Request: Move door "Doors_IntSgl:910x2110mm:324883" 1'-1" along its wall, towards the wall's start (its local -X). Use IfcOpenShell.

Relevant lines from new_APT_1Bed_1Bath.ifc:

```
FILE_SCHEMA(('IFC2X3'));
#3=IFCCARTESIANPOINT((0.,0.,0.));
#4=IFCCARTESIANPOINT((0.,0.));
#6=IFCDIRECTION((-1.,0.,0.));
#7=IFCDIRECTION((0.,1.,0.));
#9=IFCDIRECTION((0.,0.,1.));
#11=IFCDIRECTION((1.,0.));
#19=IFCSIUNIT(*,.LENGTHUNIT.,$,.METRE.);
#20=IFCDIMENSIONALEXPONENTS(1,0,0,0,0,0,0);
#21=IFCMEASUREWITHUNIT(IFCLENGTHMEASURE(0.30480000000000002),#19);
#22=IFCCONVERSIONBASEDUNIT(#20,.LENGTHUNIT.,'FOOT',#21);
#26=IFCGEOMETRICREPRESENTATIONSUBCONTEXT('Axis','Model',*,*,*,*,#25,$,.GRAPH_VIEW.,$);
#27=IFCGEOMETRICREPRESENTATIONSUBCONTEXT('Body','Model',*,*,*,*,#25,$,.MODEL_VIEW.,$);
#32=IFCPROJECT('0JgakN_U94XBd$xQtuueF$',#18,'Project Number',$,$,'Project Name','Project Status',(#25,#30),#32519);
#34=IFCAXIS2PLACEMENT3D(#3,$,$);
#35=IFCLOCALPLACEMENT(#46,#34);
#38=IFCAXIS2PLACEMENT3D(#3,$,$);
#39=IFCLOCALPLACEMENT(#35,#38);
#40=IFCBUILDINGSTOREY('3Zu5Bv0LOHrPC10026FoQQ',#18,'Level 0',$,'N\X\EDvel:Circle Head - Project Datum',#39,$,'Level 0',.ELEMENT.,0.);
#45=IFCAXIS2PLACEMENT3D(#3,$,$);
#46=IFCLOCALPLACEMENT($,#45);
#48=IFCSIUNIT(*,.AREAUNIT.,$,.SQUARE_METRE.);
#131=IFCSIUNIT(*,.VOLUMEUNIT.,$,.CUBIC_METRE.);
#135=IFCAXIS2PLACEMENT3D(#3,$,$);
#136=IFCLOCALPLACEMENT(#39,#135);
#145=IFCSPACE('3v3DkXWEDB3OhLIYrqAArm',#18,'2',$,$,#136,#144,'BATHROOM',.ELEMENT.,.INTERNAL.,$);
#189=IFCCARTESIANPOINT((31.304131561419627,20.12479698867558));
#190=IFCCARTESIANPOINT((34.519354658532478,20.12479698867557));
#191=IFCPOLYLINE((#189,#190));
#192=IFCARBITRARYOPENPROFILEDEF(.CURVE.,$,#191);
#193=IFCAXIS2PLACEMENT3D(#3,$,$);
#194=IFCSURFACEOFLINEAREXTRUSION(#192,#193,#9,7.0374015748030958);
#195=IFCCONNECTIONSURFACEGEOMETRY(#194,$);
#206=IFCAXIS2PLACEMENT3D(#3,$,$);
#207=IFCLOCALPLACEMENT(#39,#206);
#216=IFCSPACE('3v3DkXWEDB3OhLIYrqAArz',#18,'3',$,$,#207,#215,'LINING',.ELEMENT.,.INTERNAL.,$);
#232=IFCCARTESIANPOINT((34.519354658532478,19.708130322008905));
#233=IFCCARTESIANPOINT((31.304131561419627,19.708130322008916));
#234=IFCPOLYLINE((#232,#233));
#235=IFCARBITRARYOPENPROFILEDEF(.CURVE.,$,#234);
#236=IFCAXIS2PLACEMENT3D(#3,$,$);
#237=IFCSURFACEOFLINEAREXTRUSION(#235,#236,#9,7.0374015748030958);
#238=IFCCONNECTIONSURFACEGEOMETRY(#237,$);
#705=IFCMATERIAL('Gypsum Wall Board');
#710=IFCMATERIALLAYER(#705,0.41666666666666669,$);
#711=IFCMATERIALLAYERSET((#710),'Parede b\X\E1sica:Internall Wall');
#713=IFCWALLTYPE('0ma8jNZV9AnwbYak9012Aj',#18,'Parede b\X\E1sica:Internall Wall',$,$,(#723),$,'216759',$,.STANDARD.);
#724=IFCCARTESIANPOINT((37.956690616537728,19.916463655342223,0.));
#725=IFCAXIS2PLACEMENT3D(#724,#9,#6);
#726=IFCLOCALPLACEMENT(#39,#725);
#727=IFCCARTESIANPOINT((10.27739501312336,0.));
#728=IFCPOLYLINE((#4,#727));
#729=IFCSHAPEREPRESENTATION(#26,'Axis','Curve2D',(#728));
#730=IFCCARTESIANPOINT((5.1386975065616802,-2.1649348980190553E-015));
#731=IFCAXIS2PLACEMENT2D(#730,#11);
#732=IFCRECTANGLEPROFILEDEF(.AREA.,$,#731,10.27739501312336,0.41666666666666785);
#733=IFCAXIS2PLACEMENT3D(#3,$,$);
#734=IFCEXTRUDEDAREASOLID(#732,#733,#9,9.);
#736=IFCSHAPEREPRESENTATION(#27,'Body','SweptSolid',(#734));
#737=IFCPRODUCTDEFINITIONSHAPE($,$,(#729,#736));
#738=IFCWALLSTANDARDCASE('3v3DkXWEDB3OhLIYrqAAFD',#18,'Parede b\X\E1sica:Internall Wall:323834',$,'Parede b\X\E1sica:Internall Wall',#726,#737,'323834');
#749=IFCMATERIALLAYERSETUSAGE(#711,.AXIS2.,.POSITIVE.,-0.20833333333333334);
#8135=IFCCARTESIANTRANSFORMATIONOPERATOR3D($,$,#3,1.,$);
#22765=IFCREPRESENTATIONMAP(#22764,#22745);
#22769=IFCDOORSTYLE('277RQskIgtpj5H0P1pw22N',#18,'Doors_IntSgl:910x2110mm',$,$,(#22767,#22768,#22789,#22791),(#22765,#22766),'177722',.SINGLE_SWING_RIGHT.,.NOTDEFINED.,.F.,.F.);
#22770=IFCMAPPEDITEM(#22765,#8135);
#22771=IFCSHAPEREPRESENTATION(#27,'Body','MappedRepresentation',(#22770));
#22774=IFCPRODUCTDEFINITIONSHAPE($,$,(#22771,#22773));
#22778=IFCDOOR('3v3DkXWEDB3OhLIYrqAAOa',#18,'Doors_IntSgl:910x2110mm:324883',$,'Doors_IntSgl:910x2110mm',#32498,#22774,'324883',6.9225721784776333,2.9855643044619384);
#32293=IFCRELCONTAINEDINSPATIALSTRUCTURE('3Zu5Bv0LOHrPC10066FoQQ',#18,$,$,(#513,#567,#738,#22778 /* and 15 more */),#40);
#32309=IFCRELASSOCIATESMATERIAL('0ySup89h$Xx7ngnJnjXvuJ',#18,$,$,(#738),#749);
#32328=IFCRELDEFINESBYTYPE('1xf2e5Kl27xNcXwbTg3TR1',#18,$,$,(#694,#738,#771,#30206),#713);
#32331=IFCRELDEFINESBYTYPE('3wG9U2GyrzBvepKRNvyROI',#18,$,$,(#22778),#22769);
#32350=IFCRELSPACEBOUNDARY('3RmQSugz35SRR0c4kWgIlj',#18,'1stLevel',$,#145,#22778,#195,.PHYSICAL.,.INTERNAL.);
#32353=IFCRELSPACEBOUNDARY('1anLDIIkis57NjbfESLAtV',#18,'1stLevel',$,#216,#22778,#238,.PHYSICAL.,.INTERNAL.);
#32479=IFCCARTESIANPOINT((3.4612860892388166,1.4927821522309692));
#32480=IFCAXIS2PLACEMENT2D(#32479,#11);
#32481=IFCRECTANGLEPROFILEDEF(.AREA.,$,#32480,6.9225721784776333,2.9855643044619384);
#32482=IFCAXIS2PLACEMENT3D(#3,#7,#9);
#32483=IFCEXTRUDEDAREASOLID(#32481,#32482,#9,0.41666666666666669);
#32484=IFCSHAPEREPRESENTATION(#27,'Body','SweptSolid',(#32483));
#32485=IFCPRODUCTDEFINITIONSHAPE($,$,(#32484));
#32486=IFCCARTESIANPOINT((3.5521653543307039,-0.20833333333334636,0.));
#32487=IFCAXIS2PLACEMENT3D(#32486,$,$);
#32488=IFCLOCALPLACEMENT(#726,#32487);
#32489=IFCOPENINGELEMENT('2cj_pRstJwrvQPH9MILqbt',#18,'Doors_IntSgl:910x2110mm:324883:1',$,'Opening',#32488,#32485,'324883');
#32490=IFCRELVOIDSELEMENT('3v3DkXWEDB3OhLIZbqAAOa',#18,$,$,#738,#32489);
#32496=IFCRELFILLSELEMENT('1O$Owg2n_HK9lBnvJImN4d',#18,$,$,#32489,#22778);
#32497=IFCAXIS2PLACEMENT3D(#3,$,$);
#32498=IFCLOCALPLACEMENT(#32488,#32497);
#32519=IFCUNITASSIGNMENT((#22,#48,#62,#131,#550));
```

```python
import numpy as np
import ifcopenshell
import ifcopenshell.api.geometry
import ifcopenshell.util.placement
import ifcopenshell.util.unit

model = ifcopenshell.open("new_APT_1Bed_1Bath.ifc")
unit_scale = ifcopenshell.util.unit.calculate_unit_scale(model)

door = model.by_guid("3v3DkXWEDB3OhLIYrqAAOa")
opening = door.FillsVoids[0].RelatingOpeningElement
wall = opening.VoidsElements[0].RelatingBuildingElement

wall_matrix = ifcopenshell.util.placement.get_local_placement(wall.ObjectPlacement)
shift = wall_matrix[:3, 0] * -13 * 0.0254 / unit_scale
before = ifcopenshell.util.placement.get_local_placement(door.ObjectPlacement)[:3, 3].copy()

# The door is placed relative to its opening, so it follows when the opening moves.
matrix = ifcopenshell.util.placement.get_local_placement(opening.ObjectPlacement)
matrix[:3, 3] += shift
ifcopenshell.api.geometry.edit_object_placement(
    model, product=opening, matrix=matrix, is_si=False, should_transform_children=True
)

# Space boundary surfaces are stored in each space's coordinates; move them too.
for rel in door.ProvidesBoundaries:
    if not rel.ConnectionGeometry:
        continue
    surface = rel.ConnectionGeometry.SurfaceOnRelatingElement
    space_matrix = ifcopenshell.util.placement.get_local_placement(rel.RelatingSpace.ObjectPlacement)
    point = np.array(surface.Position.Location.Coordinates) + space_matrix[:3, :3].T @ shift
    surface.Position = model.createIfcAxis2Placement3D(
        model.createIfcCartesianPoint(point.tolist()), surface.Position.Axis, surface.Position.RefDirection
    )

after = ifcopenshell.util.placement.get_local_placement(door.ObjectPlacement)[:3, 3]
print("door moved by", (after - before).round(3) + 0.0)

model.write("new_APT_1Bed_1Bath_edited.ifc")
```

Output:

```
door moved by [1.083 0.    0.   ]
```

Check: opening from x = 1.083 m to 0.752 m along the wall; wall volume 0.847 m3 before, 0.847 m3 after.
